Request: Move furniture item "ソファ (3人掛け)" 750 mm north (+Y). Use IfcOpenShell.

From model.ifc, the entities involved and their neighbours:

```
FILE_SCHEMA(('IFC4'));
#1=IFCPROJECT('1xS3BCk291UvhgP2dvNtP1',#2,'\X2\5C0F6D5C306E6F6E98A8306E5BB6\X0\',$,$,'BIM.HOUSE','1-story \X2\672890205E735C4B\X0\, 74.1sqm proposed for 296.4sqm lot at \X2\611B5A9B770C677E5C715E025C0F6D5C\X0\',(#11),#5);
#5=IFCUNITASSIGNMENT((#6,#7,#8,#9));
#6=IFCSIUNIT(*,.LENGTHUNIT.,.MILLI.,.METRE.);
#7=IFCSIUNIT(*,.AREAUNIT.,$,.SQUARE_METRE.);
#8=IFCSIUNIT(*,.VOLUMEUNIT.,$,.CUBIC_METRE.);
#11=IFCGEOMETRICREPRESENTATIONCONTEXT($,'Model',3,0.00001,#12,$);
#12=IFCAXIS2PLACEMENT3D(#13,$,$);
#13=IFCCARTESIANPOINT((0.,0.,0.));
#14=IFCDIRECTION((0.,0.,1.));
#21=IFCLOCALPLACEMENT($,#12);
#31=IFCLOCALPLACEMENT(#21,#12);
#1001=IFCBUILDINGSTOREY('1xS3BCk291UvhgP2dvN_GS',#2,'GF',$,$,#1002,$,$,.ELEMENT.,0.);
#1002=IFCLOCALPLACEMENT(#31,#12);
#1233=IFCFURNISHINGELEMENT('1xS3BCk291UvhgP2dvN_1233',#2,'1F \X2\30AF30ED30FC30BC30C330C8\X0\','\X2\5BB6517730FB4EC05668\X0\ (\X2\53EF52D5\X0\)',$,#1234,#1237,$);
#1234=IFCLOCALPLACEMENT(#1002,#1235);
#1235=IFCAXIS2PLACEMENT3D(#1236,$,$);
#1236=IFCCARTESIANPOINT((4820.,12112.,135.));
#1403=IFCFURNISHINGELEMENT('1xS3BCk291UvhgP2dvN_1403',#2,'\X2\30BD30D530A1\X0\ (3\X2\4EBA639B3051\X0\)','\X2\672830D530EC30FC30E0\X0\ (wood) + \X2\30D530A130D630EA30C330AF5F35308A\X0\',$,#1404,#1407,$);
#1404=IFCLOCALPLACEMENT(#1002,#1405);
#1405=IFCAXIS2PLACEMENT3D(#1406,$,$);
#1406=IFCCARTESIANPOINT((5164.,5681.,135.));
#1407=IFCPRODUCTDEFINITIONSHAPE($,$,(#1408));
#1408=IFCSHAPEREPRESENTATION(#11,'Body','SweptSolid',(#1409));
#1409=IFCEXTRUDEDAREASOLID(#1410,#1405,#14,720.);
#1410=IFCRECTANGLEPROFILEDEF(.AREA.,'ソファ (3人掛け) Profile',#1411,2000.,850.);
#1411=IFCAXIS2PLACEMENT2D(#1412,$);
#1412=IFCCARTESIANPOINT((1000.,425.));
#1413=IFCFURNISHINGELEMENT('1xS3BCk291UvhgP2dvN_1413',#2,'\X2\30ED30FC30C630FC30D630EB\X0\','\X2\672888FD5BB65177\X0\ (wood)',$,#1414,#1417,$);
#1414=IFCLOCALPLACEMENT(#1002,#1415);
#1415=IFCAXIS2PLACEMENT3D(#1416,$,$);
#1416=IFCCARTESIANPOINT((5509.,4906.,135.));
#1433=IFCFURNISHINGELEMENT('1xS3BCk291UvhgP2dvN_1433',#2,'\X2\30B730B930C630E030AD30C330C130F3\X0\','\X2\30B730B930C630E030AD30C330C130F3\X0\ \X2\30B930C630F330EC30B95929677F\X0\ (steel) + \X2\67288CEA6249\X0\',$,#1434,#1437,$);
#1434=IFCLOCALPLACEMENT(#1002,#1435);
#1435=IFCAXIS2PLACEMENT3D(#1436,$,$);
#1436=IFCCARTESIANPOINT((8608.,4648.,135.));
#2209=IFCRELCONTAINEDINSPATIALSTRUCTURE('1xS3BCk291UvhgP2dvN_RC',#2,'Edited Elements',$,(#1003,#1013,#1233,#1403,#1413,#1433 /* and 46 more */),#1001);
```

```python
import ifcopenshell
import ifcopenshell.api.geometry
import ifcopenshell.util.placement
import ifcopenshell.util.unit

model = ifcopenshell.open("model.ifc")
unit_scale = ifcopenshell.util.unit.calculate_unit_scale(model)

item = model.by_guid("1xS3BCk291UvhgP2dvN_1403")
matrix = ifcopenshell.util.placement.get_local_placement(item.ObjectPlacement)
matrix[1, 3] += 0.75 / unit_scale
ifcopenshell.api.geometry.edit_object_placement(model, product=item, matrix=matrix, is_si=False)

print(ifcopenshell.util.placement.get_local_placement(item.ObjectPlacement).round(3) + 0.0)

model.write("model_v2.ifc")
```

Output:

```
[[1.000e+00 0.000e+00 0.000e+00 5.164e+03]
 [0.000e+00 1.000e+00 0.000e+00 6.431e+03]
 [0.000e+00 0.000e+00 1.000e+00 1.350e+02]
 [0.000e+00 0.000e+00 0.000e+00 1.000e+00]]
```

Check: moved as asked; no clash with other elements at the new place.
